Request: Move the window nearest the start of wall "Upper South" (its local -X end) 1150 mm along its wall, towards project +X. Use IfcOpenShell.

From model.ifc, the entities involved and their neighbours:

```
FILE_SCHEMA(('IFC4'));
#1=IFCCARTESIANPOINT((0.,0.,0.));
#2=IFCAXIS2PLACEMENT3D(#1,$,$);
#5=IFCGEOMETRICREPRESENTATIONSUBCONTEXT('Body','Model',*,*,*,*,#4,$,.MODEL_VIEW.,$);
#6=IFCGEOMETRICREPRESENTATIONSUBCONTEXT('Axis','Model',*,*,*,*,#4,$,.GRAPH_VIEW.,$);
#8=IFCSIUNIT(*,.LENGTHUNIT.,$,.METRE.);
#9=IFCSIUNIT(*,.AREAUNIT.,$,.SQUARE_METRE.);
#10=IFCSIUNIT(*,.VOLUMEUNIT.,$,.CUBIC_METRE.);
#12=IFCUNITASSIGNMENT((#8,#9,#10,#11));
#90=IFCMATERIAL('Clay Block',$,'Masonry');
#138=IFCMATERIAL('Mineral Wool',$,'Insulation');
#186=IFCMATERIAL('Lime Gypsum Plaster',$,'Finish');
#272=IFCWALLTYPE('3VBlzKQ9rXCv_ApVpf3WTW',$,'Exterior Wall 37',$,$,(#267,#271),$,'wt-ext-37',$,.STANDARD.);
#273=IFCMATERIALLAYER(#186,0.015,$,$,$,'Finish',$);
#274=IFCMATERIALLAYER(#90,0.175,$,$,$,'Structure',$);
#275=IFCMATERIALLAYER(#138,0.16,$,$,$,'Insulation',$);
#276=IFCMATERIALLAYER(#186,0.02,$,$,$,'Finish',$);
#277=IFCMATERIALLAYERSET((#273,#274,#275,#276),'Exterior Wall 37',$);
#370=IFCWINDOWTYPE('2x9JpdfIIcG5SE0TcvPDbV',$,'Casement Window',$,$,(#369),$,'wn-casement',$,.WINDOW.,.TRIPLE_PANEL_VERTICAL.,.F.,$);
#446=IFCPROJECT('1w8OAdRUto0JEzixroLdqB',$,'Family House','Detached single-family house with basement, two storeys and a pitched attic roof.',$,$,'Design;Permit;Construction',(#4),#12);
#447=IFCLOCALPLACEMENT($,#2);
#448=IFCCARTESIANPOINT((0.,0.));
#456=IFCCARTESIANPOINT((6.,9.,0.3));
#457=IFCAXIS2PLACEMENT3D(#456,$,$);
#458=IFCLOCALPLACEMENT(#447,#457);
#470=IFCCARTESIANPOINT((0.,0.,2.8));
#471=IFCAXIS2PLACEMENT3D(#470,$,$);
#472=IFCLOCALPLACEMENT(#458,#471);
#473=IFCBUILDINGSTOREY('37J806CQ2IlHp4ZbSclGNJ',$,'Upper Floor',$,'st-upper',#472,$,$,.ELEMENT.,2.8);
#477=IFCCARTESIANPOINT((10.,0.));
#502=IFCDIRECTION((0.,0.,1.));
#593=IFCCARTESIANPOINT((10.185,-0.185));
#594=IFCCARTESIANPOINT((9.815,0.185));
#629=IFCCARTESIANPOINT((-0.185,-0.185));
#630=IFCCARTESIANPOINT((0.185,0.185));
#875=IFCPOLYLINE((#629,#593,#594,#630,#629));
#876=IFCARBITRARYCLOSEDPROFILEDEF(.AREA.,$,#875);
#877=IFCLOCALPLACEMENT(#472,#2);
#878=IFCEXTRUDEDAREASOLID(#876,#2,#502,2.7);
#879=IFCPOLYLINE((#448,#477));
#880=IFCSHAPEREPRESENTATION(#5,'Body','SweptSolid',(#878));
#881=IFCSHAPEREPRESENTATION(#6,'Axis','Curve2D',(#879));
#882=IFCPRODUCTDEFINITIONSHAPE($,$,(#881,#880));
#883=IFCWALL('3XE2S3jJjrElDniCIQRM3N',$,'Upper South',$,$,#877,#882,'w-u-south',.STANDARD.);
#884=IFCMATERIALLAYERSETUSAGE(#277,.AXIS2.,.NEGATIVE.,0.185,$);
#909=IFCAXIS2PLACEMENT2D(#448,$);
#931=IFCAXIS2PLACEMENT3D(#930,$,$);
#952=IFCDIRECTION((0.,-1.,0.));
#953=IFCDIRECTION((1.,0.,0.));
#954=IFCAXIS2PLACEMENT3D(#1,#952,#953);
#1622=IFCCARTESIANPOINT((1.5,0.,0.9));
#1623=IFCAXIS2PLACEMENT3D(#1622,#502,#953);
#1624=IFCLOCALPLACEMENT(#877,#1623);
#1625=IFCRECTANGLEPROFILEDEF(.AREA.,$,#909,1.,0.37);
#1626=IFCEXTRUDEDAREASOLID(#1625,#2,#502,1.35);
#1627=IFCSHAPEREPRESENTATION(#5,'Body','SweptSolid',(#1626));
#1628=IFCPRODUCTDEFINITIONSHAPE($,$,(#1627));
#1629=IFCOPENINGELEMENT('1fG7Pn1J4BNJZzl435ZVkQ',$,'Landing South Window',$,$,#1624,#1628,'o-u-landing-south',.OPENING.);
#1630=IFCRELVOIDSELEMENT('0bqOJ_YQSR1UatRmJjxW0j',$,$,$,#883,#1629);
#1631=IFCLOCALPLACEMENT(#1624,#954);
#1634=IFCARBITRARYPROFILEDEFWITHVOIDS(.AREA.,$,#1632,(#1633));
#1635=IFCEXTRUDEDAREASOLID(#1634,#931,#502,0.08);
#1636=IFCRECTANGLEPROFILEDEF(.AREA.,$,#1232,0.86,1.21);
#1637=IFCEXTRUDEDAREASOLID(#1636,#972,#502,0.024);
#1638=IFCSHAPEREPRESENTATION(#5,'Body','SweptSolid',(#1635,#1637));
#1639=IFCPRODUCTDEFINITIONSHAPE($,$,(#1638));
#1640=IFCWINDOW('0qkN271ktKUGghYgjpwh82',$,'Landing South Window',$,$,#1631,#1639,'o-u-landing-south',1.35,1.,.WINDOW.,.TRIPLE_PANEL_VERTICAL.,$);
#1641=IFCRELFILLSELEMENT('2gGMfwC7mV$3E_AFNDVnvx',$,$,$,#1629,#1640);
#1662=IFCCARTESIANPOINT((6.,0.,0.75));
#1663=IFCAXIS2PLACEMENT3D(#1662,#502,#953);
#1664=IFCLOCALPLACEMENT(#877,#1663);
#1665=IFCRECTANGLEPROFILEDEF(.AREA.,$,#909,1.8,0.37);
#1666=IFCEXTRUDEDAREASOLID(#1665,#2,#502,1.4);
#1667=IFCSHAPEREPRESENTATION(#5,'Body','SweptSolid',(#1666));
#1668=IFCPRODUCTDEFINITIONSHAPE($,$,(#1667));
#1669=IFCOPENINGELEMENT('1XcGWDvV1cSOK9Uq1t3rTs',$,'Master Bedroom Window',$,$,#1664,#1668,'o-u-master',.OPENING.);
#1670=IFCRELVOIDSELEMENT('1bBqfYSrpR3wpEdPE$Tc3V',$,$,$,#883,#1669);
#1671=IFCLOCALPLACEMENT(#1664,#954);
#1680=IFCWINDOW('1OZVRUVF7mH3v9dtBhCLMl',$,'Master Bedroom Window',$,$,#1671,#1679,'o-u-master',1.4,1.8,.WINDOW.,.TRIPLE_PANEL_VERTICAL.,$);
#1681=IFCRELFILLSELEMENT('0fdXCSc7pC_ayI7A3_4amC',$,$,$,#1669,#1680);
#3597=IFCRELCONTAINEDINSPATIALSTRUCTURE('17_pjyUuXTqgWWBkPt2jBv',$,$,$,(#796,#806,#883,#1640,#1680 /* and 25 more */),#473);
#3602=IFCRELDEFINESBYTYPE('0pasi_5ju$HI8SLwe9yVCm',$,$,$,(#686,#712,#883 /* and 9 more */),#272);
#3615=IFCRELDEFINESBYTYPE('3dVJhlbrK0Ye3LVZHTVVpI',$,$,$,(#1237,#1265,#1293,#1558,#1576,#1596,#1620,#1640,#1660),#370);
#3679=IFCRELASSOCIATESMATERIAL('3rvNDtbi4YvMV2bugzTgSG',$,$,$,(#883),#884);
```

```python
import ifcopenshell
import ifcopenshell.api.geometry
import ifcopenshell.util.placement
import ifcopenshell.util.unit

model = ifcopenshell.open("model.ifc")
unit_scale = ifcopenshell.util.unit.calculate_unit_scale(model)

window = model.by_id(1640)
opening = window.FillsVoids[0].RelatingOpeningElement
wall = opening.VoidsElements[0].RelatingBuildingElement

wall_matrix = ifcopenshell.util.placement.get_local_placement(wall.ObjectPlacement)
shift = wall_matrix[:3, 0] * 1.15 / unit_scale
before = ifcopenshell.util.placement.get_local_placement(window.ObjectPlacement)[:3, 3].copy()

# The window is placed relative to its opening, so it follows when the opening moves.
matrix = ifcopenshell.util.placement.get_local_placement(opening.ObjectPlacement)
matrix[:3, 3] += shift
ifcopenshell.api.geometry.edit_object_placement(
    model, product=opening, matrix=matrix, is_si=False, should_transform_children=True
)

after = ifcopenshell.util.placement.get_local_placement(window.ObjectPlacement)[:3, 3]
print("window moved by", (after - before).round(3) + 0.0)

model.write("model_rev.ifc")
```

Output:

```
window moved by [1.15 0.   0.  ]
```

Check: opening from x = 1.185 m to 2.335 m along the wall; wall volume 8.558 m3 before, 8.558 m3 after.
